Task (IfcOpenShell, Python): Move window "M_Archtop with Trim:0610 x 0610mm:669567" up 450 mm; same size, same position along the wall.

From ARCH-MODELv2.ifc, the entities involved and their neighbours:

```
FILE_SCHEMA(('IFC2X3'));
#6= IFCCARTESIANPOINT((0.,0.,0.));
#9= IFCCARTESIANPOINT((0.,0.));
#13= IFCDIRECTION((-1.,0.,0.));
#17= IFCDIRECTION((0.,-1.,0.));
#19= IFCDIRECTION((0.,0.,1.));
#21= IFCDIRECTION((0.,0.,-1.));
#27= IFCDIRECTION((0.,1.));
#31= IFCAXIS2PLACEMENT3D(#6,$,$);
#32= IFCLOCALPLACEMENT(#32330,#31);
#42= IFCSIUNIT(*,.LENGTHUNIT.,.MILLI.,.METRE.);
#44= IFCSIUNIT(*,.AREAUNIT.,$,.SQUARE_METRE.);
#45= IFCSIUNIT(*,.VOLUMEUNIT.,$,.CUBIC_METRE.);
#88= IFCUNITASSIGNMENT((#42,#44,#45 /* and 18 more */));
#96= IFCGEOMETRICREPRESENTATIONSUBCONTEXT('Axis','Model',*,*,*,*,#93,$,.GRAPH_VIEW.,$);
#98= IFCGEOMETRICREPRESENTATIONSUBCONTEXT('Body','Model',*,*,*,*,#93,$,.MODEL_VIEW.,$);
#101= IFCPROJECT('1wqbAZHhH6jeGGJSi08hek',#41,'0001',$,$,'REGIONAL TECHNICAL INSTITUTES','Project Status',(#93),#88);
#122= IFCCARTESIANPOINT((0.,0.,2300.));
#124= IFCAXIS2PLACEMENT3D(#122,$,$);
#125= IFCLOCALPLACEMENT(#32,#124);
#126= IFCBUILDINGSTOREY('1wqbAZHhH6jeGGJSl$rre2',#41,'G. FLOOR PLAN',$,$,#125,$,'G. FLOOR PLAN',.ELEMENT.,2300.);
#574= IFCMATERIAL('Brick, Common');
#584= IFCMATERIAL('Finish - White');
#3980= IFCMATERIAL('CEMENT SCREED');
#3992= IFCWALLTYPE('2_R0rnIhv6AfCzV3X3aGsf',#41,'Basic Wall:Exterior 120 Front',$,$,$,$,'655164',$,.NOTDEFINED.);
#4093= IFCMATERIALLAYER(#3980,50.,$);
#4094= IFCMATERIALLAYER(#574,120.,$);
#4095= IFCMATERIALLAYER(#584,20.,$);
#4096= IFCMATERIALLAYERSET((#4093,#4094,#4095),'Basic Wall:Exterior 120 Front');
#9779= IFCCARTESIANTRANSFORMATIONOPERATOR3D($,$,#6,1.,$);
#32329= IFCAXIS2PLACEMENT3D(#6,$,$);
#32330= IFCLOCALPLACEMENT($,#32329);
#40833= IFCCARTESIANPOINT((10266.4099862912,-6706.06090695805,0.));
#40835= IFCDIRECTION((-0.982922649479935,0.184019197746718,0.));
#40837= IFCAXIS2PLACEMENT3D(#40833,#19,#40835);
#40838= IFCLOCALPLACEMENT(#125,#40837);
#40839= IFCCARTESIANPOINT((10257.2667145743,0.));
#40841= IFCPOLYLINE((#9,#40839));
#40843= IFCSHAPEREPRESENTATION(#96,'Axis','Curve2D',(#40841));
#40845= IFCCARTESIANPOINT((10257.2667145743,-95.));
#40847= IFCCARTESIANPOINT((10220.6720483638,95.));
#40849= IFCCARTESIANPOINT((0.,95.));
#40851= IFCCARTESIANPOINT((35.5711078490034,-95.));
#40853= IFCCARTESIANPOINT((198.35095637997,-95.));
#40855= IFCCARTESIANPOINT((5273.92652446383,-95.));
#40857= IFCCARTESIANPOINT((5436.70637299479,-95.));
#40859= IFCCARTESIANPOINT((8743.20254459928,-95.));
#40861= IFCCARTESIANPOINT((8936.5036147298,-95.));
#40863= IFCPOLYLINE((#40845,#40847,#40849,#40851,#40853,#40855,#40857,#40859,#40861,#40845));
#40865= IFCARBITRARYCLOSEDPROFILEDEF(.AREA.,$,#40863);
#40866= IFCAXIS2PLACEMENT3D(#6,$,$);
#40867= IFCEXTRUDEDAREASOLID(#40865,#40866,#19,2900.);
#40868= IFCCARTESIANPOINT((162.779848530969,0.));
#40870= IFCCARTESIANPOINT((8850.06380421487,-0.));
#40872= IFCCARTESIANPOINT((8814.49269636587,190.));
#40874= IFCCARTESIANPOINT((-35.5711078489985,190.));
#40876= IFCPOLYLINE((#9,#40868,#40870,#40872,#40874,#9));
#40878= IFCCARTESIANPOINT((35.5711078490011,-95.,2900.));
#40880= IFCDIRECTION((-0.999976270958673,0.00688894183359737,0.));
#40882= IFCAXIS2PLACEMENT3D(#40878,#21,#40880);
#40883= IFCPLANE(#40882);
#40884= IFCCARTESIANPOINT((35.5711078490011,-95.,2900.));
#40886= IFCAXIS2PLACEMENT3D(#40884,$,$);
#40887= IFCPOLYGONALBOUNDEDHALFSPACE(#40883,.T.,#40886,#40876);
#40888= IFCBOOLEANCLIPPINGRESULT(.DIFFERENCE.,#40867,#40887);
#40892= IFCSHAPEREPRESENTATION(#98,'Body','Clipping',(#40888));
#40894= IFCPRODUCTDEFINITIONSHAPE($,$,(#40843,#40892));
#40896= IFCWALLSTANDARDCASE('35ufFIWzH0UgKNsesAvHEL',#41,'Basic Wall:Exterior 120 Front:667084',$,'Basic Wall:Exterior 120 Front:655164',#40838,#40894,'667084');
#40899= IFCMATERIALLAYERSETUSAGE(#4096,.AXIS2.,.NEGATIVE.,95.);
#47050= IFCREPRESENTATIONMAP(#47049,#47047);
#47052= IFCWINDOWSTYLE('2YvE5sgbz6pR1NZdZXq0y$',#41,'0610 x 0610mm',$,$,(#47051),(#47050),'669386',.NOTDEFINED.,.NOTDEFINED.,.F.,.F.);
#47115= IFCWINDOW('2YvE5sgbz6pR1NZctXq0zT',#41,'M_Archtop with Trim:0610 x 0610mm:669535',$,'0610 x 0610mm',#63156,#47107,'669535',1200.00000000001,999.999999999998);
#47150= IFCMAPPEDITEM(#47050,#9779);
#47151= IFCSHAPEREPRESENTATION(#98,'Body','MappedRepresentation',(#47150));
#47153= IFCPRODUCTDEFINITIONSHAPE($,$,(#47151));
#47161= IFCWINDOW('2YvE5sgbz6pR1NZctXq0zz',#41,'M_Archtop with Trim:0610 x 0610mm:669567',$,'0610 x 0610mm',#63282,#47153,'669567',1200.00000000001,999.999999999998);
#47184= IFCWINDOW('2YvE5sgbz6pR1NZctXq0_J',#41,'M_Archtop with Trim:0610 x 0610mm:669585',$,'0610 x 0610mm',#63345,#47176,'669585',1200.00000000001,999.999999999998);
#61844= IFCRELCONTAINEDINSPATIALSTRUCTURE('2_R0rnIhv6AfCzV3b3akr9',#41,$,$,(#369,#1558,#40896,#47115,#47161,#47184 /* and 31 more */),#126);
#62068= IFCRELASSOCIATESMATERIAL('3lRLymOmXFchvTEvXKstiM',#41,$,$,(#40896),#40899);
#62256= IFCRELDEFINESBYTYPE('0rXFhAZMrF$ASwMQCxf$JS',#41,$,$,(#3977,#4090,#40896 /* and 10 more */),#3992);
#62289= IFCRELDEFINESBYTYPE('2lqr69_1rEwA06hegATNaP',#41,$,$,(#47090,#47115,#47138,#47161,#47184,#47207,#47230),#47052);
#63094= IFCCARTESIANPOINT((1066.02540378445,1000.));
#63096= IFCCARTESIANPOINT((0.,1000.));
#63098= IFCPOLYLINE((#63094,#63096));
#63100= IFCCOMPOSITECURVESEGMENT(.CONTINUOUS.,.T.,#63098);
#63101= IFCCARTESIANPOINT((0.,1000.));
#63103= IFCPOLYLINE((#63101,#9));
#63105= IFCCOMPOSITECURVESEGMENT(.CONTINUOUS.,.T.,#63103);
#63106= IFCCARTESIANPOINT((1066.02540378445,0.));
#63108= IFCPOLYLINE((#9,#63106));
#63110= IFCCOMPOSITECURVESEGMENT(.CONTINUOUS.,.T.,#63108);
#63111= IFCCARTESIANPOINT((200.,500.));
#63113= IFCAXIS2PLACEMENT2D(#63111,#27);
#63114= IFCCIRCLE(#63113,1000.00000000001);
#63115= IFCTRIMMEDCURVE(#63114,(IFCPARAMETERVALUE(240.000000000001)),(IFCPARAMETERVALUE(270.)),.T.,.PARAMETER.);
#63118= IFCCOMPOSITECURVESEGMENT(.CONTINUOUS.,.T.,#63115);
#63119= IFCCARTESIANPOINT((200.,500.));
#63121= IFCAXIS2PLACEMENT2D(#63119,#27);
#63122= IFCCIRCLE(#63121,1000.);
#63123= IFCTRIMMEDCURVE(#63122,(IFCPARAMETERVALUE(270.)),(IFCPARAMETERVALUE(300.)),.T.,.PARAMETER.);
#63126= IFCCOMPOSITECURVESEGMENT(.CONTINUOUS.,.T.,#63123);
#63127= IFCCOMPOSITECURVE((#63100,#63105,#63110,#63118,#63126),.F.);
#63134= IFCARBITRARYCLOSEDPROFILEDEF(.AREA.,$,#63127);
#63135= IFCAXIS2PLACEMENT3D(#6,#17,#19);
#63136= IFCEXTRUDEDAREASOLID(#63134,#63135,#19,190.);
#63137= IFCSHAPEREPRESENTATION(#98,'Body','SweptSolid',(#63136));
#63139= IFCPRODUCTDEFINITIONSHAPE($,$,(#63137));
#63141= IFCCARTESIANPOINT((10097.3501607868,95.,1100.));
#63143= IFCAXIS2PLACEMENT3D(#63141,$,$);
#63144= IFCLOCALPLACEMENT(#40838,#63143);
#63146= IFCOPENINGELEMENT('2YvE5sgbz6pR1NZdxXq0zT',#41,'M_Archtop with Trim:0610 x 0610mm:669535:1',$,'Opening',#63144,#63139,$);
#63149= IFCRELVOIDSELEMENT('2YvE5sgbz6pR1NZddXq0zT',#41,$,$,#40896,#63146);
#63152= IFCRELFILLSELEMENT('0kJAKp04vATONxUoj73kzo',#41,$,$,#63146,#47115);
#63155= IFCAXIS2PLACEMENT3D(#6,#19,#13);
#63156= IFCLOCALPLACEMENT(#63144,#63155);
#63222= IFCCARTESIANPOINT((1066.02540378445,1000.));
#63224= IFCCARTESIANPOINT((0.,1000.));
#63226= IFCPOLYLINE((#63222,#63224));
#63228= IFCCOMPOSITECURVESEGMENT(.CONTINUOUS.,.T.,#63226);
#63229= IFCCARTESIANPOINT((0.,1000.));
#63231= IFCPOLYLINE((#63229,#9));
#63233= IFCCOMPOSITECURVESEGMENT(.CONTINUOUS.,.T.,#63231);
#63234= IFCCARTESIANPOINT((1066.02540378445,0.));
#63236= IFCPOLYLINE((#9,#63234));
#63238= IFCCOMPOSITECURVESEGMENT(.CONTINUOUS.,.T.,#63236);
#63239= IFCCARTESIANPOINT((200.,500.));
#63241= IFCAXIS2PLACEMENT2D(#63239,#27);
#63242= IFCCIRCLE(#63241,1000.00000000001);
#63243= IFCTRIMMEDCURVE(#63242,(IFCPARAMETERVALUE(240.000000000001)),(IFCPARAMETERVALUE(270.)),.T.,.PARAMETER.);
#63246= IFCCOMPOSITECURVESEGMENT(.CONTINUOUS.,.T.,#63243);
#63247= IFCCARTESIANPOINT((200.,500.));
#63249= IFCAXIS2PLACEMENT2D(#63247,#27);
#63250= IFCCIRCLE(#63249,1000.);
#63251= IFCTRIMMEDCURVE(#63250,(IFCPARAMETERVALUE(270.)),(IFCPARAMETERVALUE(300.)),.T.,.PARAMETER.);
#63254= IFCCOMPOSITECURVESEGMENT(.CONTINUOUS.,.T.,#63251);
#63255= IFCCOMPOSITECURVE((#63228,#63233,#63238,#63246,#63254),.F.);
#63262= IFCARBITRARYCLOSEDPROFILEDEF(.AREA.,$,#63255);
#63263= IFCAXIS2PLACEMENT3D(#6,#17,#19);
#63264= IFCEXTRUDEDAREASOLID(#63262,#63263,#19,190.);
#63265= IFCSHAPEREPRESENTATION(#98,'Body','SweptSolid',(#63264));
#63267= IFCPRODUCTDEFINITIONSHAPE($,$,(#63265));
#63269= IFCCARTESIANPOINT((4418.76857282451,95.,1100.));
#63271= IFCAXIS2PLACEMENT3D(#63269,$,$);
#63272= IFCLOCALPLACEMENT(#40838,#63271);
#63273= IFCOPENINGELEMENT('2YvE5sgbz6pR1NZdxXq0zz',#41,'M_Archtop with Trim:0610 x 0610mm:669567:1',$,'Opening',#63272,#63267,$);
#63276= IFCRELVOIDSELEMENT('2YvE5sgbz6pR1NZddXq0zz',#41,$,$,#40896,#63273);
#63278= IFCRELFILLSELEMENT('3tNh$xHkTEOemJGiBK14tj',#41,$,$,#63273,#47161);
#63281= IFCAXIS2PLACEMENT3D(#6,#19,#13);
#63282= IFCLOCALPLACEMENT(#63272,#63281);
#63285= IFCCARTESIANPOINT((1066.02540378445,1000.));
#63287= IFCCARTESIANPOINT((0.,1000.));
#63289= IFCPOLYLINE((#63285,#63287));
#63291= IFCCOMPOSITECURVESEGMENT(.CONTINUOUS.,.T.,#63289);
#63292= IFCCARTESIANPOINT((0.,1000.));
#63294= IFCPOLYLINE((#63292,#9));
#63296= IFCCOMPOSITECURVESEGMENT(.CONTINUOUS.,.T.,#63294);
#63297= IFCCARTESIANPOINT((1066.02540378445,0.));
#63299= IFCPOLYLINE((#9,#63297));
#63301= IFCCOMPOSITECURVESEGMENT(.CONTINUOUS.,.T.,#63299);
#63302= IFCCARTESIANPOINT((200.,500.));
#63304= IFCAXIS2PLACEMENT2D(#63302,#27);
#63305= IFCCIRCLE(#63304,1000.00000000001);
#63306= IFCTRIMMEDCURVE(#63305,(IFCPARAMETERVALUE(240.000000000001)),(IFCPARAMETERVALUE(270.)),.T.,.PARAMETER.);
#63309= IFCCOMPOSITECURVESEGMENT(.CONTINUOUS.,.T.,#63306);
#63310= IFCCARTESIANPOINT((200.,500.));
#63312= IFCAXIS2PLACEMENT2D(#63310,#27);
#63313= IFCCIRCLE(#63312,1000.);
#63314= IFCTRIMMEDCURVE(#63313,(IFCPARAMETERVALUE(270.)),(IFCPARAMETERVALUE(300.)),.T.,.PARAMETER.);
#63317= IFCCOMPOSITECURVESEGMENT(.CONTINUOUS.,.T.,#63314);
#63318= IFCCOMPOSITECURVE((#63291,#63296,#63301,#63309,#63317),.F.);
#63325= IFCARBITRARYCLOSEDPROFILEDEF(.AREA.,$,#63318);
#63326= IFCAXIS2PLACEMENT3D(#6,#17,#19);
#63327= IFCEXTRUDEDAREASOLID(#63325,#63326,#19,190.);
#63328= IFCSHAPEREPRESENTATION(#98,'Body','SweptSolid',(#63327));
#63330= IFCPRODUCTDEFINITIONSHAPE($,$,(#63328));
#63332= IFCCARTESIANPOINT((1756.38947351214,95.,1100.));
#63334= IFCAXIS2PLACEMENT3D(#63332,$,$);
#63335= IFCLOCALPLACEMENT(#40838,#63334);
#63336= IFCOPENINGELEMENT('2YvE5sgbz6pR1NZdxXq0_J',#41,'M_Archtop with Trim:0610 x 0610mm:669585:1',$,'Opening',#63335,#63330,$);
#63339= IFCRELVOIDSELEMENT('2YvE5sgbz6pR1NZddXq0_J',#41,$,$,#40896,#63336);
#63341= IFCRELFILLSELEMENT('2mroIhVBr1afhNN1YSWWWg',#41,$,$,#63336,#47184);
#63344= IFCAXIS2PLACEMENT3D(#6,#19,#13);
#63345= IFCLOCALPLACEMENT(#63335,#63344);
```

```python
import numpy as np
import ifcopenshell
import ifcopenshell.api.geometry
import ifcopenshell.util.placement
import ifcopenshell.util.unit

model = ifcopenshell.open("ARCH-MODELv2.ifc")
unit_scale = ifcopenshell.util.unit.calculate_unit_scale(model)

window = model.by_guid("2YvE5sgbz6pR1NZctXq0zz")
opening = window.FillsVoids[0].RelatingOpeningElement
dz = 0.45 / unit_scale

shift = np.array([0.0, 0.0, dz])
# The window is placed relative to its opening, so it follows when the opening moves.
matrix = ifcopenshell.util.placement.get_local_placement(opening.ObjectPlacement)
matrix[:3, 3] += shift
ifcopenshell.api.geometry.edit_object_placement(
    model, product=opening, matrix=matrix, is_si=False, should_transform_children=True
)

print(f"moved by {dz * unit_scale:+.3f} m")

model.write("ARCH-MODELv2-out.ifc")
```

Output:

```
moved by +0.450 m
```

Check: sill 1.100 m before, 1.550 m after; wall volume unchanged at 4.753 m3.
